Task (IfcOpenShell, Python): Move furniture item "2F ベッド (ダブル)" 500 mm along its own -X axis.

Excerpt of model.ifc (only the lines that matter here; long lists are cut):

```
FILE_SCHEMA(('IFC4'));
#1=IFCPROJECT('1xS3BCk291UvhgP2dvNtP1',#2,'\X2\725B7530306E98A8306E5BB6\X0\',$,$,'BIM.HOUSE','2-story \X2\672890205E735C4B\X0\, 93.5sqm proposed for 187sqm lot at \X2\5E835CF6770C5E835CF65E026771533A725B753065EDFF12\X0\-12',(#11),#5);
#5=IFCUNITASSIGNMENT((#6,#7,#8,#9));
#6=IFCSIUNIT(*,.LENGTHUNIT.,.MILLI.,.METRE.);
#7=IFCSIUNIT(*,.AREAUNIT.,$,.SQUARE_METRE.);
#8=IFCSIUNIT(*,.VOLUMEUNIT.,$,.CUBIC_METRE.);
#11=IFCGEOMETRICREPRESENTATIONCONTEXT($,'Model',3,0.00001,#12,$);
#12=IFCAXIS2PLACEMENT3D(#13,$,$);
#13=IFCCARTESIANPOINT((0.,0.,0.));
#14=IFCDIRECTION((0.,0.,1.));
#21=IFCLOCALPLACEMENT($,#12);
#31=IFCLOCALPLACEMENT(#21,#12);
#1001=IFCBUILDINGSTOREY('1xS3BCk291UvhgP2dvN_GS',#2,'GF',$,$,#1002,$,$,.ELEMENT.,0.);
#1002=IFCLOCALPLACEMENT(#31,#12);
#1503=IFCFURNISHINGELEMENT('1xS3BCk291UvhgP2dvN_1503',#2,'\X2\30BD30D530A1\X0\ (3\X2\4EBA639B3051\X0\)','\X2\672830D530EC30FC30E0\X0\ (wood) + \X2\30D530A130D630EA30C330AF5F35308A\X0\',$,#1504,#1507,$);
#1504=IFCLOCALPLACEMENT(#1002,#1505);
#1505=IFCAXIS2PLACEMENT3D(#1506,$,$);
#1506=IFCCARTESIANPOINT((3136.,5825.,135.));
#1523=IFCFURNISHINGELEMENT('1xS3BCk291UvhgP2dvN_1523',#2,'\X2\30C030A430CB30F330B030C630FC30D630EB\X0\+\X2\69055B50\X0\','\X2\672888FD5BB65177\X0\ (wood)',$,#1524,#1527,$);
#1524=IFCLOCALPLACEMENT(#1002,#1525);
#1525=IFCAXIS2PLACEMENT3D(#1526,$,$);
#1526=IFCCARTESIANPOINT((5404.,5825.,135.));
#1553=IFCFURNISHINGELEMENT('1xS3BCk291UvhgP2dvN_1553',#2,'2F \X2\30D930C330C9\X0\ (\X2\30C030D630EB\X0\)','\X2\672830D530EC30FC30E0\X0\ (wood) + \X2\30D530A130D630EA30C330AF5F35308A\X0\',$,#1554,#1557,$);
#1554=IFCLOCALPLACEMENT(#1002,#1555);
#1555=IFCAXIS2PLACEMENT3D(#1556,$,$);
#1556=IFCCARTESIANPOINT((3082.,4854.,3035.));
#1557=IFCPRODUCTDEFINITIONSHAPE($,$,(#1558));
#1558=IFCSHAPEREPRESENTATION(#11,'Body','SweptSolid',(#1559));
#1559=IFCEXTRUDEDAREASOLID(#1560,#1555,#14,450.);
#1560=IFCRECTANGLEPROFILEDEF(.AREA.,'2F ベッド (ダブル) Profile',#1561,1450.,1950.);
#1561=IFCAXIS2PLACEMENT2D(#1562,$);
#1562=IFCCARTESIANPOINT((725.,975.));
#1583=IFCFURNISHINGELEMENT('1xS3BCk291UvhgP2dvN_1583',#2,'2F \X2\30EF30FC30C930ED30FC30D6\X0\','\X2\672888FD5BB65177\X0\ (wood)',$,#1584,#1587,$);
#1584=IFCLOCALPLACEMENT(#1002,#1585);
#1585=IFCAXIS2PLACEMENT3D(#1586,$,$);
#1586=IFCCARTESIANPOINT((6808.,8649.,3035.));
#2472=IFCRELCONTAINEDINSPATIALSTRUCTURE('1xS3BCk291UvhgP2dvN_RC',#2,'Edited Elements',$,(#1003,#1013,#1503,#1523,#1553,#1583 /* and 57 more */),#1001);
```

```python
import ifcopenshell
import ifcopenshell.api.geometry
import ifcopenshell.util.placement
import ifcopenshell.util.unit

model = ifcopenshell.open("model.ifc")
unit_scale = ifcopenshell.util.unit.calculate_unit_scale(model)

item = model.by_id(1553)
matrix = ifcopenshell.util.placement.get_local_placement(item.ObjectPlacement)
matrix[:3, 3] -= matrix[:3, 0] * 0.5 / unit_scale
ifcopenshell.api.geometry.edit_object_placement(model, product=item, matrix=matrix, is_si=False)

print(ifcopenshell.util.placement.get_local_placement(item.ObjectPlacement).round(3) + 0.0)

model.write("model_rev.ifc")
```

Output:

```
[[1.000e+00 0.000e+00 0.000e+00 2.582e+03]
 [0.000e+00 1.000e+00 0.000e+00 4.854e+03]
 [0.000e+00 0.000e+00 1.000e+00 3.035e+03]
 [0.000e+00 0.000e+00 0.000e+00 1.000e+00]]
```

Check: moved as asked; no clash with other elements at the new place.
